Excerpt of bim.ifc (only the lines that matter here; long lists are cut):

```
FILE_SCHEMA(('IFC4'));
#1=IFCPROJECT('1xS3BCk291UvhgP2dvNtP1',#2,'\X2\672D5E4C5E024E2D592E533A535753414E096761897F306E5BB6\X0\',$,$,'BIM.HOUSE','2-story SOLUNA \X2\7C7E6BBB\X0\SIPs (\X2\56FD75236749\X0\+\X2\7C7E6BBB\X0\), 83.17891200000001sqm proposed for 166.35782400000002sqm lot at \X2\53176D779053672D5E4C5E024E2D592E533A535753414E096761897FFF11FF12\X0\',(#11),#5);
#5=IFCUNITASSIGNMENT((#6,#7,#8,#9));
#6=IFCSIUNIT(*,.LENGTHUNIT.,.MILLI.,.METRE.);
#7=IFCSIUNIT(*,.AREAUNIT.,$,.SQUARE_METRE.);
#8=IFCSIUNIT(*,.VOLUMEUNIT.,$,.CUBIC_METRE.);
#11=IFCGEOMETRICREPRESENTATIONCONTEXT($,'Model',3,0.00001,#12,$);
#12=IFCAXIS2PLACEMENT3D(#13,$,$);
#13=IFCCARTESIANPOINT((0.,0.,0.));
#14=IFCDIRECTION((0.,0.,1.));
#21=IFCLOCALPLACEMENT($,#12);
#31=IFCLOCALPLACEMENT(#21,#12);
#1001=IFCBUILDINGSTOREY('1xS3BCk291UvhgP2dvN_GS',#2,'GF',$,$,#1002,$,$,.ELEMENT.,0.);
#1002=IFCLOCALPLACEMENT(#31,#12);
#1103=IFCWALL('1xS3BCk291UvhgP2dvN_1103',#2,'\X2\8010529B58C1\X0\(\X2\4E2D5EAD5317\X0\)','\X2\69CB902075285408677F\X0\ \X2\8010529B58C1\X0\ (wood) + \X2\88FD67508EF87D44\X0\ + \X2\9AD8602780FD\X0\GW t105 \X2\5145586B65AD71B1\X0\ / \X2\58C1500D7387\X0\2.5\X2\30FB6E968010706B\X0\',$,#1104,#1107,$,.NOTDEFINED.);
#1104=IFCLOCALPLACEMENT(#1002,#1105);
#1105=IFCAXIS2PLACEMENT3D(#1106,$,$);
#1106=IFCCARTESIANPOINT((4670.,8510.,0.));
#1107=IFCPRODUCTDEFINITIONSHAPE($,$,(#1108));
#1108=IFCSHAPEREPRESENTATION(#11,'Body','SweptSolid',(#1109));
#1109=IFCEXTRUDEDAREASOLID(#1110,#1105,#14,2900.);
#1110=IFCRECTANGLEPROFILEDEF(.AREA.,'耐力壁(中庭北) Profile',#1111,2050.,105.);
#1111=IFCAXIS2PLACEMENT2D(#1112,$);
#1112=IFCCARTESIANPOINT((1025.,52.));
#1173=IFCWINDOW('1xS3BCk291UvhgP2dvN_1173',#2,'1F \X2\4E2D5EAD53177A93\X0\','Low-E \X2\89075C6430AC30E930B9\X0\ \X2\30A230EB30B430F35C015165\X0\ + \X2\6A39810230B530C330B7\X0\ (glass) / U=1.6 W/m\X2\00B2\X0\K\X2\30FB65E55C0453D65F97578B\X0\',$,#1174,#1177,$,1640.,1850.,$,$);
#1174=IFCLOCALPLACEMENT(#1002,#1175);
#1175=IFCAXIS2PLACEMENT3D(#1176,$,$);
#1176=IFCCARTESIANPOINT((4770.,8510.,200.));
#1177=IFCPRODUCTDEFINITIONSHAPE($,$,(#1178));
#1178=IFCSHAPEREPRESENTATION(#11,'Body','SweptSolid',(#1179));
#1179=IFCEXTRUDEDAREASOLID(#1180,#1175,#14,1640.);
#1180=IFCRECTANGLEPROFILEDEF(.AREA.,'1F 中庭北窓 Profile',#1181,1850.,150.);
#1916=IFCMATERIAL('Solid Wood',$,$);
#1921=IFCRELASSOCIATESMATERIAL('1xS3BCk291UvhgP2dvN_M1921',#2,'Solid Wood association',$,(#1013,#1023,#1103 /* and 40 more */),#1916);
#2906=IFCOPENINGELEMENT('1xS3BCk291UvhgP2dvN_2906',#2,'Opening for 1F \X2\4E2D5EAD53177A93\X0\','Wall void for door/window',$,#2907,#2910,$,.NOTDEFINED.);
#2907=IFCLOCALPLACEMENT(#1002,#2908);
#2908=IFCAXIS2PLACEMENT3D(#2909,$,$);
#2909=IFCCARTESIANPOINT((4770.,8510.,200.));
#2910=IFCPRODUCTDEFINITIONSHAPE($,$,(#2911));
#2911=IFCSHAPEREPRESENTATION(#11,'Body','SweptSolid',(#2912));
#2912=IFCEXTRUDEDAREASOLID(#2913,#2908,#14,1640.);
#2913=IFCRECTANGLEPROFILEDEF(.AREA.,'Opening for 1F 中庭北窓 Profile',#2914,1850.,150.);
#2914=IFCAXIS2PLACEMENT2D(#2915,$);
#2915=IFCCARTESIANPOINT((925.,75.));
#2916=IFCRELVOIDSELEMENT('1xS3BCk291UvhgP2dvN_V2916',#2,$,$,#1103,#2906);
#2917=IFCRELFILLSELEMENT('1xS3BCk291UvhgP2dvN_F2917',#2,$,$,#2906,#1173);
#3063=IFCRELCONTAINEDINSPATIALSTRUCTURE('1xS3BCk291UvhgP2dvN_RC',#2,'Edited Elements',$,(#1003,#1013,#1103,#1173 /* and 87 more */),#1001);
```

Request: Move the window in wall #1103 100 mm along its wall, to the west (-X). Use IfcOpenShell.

```python
import ifcopenshell
import ifcopenshell.api.geometry
import ifcopenshell.util.placement
import ifcopenshell.util.unit

model = ifcopenshell.open("bim.ifc")
unit_scale = ifcopenshell.util.unit.calculate_unit_scale(model)

window = model.by_id(1173)
opening = window.FillsVoids[0].RelatingOpeningElement
wall = opening.VoidsElements[0].RelatingBuildingElement

wall_matrix = ifcopenshell.util.placement.get_local_placement(wall.ObjectPlacement)
shift = wall_matrix[:3, 0] * -0.1 / unit_scale
before = ifcopenshell.util.placement.get_local_placement(window.ObjectPlacement)[:3, 3].copy()

# The window is not placed relative to its opening, so move both.
for product in (opening, window):
    matrix = ifcopenshell.util.placement.get_local_placement(product.ObjectPlacement)
    matrix[:3, 3] += shift
    ifcopenshell.api.geometry.edit_object_placement(model, product=product, matrix=matrix, is_si=False)

after = ifcopenshell.util.placement.get_local_placement(window.ObjectPlacement)[:3, 3]
print("window moved by", (after - before).round(3) + 0.0)

model.write("bim_edited.ifc")
```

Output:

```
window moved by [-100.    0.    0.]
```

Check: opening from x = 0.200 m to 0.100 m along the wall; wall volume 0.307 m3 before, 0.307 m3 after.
